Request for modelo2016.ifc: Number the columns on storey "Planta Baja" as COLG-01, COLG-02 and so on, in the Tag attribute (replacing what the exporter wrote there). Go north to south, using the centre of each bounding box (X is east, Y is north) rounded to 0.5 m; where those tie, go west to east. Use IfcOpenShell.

First a look at what the model holds.

```python
import ifcopenshell
import ifcopenshell.util.element
import ifcopenshell.util.placement

model = ifcopenshell.open("modelo2016.ifc")
print(model.schema)
storey = next(s for s in model.by_type("IfcBuildingStorey") if s.Name == "Planta Baja")
columns = [e for e in ifcopenshell.util.element.get_decomposition(storey) if e.is_a("IfcColumn")]
for e in sorted(columns, key=lambda e: e.id()):
    origin = ifcopenshell.util.placement.get_local_placement(e.ObjectPlacement)[:3, 3]
    print(e.id(), e.Tag, e.Name, origin.round(2) + 0.0, sep=" | ")
```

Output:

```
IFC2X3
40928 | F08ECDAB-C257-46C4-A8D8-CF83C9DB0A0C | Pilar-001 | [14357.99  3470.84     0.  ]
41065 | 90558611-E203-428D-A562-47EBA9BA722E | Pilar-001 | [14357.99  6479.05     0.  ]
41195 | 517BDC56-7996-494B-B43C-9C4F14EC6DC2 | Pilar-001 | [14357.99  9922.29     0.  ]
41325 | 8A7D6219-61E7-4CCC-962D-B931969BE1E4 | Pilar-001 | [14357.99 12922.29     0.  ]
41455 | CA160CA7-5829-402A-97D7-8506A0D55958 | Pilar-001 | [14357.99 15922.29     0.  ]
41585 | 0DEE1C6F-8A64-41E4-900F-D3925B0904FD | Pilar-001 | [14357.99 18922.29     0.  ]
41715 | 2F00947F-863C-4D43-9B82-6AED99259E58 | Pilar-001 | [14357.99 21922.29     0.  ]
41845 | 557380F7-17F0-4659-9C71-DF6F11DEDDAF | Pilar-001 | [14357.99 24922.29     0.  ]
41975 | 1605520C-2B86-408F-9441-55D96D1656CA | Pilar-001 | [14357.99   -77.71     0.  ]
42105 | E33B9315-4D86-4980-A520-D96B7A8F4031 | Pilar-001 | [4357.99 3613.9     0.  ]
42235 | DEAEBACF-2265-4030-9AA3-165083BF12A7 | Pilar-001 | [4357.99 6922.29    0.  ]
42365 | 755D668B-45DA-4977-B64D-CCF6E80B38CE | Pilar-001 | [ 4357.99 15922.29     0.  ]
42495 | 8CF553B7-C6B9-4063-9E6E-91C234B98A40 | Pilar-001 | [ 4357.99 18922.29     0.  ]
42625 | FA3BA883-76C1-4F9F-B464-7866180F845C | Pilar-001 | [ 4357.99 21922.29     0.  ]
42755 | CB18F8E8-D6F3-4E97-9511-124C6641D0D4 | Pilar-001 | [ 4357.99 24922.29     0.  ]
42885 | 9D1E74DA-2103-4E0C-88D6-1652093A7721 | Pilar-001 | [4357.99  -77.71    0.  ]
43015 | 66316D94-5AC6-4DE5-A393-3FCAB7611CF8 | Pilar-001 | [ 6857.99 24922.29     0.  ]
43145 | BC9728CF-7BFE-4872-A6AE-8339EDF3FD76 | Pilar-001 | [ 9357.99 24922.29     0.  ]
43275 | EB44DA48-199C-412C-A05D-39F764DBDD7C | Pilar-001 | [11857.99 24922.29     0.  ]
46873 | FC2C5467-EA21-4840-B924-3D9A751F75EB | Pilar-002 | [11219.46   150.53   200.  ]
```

```python
import ifcopenshell
import ifcopenshell.geom
import ifcopenshell.util.element
import ifcopenshell.util.shape

model = ifcopenshell.open("modelo2016.ifc")
settings = ifcopenshell.geom.settings()
settings.set("use-world-coords", True)


def centre(element):
    shape = ifcopenshell.geom.create_shape(settings, element)
    return ifcopenshell.util.shape.get_bbox_centroid(shape.geometry)


storey = next(s for s in model.by_type("IfcBuildingStorey") if s.Name == "Planta Baja")
columns = [e for e in ifcopenshell.util.element.get_decomposition(storey) if e.is_a("IfcColumn")]

# Insertion points can sit at a corner or the storey origin, so sort by the geometry (in metres).
centres = {e: centre(e) for e in columns}
columns.sort(key=lambda e: (-round(centres[e][1] / 0.5), centres[e][0]))

for i, e in enumerate(columns, start=1):
    number = f"COLG-{i:02d}"
    e.Tag = number
    print(e.id(), number)

model.write("modelo2016_edited.ifc")
```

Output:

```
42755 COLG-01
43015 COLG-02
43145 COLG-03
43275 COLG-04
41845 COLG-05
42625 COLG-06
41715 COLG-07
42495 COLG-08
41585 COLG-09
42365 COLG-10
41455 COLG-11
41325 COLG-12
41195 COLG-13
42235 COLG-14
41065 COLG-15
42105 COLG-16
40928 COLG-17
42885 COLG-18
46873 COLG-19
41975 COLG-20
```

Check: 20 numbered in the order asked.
